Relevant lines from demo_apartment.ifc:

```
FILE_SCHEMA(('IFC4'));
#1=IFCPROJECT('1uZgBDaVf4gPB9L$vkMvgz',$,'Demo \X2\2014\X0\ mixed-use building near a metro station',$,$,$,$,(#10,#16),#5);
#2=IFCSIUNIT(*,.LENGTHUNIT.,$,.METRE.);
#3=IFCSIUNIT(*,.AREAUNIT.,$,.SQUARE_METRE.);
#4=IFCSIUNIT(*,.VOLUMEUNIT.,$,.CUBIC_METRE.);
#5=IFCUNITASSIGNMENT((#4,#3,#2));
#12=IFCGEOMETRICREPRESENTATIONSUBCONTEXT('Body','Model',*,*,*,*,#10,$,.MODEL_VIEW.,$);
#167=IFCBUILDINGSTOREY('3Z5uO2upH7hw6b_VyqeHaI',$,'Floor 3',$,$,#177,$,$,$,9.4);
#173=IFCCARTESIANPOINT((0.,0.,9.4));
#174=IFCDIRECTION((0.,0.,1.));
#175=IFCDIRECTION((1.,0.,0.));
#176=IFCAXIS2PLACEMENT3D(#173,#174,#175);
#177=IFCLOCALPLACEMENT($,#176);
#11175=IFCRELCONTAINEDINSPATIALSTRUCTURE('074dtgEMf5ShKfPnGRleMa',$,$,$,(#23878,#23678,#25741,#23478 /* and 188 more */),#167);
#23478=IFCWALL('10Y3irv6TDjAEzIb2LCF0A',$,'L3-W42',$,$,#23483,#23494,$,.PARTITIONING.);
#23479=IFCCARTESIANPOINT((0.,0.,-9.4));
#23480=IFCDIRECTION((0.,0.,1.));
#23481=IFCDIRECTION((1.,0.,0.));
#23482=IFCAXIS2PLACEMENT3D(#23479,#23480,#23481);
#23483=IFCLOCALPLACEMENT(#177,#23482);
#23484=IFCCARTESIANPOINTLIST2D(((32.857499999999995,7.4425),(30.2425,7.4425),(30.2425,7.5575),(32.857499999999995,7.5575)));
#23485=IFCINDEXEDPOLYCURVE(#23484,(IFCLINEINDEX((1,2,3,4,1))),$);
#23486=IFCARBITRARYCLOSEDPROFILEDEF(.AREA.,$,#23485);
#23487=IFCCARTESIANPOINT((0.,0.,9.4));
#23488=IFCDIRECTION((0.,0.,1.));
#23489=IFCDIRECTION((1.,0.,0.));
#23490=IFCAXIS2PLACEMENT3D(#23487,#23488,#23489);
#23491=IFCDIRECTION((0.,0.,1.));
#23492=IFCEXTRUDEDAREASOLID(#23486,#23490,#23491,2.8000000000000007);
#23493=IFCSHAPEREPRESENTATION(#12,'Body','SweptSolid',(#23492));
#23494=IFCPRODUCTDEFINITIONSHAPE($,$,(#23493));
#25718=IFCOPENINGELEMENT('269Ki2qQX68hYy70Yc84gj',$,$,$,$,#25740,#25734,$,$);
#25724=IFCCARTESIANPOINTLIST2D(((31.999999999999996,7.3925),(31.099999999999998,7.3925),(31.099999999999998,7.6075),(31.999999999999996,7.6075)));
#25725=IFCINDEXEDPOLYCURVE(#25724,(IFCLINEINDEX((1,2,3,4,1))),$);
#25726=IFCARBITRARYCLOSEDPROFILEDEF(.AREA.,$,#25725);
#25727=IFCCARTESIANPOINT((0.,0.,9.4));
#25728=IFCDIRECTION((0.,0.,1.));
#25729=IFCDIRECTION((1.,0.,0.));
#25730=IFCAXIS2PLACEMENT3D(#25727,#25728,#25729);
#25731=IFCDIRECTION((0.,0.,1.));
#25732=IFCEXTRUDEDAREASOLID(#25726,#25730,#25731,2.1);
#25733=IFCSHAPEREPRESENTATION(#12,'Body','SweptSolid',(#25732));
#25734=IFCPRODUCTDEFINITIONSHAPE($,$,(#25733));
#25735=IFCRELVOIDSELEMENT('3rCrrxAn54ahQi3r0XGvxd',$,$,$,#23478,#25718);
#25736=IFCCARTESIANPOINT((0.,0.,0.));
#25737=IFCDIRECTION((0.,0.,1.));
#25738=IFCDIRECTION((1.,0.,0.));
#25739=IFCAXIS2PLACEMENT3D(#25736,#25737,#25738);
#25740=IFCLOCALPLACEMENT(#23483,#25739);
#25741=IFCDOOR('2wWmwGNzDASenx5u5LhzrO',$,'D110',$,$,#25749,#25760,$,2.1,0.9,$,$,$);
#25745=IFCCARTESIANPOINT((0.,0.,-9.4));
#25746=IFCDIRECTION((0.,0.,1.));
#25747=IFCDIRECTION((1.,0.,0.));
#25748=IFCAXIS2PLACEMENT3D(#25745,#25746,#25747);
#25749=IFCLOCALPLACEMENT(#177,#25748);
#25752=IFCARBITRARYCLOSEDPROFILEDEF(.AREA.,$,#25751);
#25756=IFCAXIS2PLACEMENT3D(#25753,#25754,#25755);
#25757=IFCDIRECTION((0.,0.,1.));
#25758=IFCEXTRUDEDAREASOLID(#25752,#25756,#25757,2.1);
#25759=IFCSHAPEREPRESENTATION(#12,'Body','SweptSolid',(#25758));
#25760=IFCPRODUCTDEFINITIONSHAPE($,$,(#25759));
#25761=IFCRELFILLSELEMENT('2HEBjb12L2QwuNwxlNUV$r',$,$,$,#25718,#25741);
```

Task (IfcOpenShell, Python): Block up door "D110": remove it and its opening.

```python
import ifcopenshell
import ifcopenshell.api.feature
import ifcopenshell.api.root
import ifcopenshell.geom
import ifcopenshell.util.shape

model = ifcopenshell.open("demo_apartment.ifc")
settings = ifcopenshell.geom.settings()


def volume(element):
    """Net volume in cubic metres, openings subtracted."""
    shape = ifcopenshell.geom.create_shape(settings, element)
    return ifcopenshell.util.shape.get_volume(shape.geometry)


door = model.by_id(25741)
opening = door.FillsVoids[0].RelatingOpeningElement
wall = opening.VoidsElements[0].RelatingBuildingElement
before = volume(wall)

ifcopenshell.api.root.remove_product(model, product=door)
ifcopenshell.api.feature.remove_feature(model, feature=opening)

after = volume(wall)

print(f"wall volume {before:.3f} -> {after:.3f} m3")

model.write("demo_apartment_v2.ifc")
```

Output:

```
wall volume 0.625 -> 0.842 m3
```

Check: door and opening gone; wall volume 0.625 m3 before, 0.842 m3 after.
